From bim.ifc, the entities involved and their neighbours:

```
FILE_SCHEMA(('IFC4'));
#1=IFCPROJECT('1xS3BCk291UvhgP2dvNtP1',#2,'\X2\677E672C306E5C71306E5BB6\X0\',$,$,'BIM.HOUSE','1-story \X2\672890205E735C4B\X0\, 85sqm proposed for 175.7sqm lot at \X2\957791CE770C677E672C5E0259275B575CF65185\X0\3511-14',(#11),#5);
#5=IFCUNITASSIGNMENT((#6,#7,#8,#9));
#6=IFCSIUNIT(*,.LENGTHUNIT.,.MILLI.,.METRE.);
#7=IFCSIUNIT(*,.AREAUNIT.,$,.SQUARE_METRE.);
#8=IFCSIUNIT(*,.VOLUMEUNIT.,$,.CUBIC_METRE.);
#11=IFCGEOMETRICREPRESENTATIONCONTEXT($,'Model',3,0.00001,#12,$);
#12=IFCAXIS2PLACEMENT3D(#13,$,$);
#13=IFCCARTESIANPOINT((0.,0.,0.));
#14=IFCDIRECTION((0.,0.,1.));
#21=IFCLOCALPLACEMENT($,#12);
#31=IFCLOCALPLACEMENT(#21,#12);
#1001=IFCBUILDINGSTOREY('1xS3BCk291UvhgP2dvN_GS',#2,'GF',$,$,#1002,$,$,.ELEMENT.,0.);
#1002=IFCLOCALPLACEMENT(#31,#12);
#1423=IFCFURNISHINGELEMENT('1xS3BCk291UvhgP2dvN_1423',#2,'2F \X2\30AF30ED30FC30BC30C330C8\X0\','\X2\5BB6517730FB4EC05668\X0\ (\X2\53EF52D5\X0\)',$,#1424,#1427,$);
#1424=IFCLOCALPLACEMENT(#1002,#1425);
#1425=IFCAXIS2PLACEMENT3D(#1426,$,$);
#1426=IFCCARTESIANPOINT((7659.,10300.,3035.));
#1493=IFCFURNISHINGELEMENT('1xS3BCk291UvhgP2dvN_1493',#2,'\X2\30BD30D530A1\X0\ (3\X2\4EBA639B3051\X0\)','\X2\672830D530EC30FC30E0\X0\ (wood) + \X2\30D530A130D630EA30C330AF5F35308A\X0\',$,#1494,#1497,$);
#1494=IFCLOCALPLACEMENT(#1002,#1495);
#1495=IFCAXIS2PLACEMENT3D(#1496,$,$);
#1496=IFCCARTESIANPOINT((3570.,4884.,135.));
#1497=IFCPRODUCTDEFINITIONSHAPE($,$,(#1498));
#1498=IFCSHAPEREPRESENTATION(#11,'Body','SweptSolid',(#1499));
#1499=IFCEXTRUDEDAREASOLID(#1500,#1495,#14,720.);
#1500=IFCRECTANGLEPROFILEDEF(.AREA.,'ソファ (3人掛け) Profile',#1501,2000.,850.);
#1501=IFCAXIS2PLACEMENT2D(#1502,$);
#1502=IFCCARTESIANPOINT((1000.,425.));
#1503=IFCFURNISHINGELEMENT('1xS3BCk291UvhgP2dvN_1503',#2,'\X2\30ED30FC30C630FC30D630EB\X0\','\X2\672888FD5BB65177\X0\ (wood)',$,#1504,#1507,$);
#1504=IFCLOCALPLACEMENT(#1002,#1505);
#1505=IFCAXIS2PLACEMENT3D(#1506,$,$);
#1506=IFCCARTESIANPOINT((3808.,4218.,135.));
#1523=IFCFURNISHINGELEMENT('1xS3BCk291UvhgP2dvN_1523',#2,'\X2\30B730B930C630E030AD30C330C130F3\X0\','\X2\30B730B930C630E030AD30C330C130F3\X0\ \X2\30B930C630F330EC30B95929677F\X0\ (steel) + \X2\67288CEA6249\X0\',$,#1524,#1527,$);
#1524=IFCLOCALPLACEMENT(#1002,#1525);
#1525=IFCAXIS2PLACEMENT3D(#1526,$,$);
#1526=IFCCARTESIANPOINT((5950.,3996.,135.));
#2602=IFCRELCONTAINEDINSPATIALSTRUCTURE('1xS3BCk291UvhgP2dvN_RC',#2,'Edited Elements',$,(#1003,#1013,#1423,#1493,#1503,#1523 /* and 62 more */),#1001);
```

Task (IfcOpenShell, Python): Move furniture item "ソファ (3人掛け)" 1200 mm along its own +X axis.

```python
import ifcopenshell
import ifcopenshell.api.geometry
import ifcopenshell.util.placement
import ifcopenshell.util.unit

model = ifcopenshell.open("bim.ifc")
unit_scale = ifcopenshell.util.unit.calculate_unit_scale(model)

item = model.by_guid("1xS3BCk291UvhgP2dvN_1493")
matrix = ifcopenshell.util.placement.get_local_placement(item.ObjectPlacement)
matrix[:3, 3] += matrix[:3, 0] * 1.2 / unit_scale
ifcopenshell.api.geometry.edit_object_placement(model, product=item, matrix=matrix, is_si=False)

print(ifcopenshell.util.placement.get_local_placement(item.ObjectPlacement).round(3) + 0.0)

model.write("bim-out.ifc")
```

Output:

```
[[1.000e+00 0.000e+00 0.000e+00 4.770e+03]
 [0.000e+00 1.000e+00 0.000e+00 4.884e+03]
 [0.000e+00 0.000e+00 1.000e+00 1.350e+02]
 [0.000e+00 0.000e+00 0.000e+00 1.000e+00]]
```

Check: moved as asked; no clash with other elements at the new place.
